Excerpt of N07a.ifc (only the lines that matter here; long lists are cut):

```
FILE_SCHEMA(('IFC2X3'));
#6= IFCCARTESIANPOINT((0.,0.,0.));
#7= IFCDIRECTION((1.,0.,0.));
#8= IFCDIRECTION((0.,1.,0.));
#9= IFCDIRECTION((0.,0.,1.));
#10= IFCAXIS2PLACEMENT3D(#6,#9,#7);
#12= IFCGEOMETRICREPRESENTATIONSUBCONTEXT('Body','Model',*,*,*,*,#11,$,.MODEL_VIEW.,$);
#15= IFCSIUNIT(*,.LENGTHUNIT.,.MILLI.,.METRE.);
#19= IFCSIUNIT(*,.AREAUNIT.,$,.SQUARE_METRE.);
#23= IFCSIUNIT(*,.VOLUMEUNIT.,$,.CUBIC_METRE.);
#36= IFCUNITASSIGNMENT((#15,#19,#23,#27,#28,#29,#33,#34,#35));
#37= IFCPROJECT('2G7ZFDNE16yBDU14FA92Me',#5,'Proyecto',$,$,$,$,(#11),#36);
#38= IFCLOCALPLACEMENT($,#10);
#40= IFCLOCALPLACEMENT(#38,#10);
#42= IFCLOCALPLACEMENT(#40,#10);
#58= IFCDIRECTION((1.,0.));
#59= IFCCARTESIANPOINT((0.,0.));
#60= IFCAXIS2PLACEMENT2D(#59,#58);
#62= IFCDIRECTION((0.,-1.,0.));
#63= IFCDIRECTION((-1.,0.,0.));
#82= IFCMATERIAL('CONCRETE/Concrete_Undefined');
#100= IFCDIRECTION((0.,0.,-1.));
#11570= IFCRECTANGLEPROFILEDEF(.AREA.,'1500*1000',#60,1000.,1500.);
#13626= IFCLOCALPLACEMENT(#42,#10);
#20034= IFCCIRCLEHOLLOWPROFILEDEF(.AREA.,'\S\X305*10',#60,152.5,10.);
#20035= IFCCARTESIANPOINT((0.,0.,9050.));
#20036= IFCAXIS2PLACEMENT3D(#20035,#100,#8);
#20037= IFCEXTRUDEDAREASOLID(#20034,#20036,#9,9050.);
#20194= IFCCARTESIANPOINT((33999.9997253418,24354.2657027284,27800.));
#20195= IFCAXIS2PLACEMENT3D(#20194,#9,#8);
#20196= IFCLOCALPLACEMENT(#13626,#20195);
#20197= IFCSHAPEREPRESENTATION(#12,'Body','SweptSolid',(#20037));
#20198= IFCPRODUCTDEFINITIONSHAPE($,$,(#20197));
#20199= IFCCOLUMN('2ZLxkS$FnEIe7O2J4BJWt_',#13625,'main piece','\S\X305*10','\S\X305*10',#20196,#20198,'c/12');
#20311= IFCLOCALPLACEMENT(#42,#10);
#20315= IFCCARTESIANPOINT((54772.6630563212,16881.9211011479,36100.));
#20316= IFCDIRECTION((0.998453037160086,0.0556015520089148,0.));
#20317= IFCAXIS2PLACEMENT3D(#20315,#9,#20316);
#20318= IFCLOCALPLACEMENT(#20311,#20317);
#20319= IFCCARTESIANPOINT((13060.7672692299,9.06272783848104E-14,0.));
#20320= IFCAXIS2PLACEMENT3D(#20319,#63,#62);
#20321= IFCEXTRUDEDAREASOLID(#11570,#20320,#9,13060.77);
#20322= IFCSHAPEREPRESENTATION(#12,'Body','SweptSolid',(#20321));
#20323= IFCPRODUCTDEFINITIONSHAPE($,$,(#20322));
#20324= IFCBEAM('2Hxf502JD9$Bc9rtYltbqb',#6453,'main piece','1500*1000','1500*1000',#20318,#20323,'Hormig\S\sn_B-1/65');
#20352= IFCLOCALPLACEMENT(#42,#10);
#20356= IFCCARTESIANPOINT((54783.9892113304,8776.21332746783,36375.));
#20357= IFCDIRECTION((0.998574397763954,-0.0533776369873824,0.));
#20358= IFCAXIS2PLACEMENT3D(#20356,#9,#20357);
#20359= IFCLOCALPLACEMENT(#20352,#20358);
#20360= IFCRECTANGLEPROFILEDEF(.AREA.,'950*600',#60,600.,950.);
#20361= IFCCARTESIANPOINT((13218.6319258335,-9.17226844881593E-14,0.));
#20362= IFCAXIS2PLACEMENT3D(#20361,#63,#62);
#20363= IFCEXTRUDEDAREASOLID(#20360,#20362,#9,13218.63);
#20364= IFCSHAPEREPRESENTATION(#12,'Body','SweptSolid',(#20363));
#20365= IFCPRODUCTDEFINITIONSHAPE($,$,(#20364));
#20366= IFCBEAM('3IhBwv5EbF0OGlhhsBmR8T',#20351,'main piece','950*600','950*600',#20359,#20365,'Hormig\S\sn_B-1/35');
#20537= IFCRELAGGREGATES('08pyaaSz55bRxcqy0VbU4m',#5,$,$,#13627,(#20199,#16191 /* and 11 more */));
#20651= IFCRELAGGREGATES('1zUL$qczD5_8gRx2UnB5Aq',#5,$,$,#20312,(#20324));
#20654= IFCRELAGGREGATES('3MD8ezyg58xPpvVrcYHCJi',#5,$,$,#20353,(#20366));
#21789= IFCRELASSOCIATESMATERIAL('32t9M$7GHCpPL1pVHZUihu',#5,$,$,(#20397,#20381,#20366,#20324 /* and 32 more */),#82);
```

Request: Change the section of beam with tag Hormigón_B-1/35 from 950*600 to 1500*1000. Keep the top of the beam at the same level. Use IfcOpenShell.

```python
import ifcopenshell
import ifcopenshell.util.element
import ifcopenshell.util.representation

model = ifcopenshell.open("N07a.ifc")

member = model.by_guid("3IhBwv5EbF0OGlhhsBmR8T")
source = next(p for p in model.by_type("IfcRectangleProfileDef") if p.ProfileName == "1500*1000")

body = ifcopenshell.util.representation.get_representation(member, "Model", "Body")
solid = body.Items[0]
old_profile = solid.SweptArea

# Copy the section's sizes but keep this member's own profile position.
profile = ifcopenshell.util.element.copy(model, source)
# Profiles are centred, so shift by half the change in depth to hold the top.
shift = (old_profile.YDim - profile.YDim) / 2
x, y = old_profile.Position.Location.Coordinates
up = (0.0, 1.0)  # upwards, in the solid's own plane
location = model.createIfcCartesianPoint((x + up[0] * shift, y + up[1] * shift))
profile.Position = model.createIfcAxis2Placement2D(location, old_profile.Position.RefDirection)
solid.SweptArea = profile
if not model.get_total_inverses(old_profile):
    ifcopenshell.util.element.remove_deep2(model, old_profile)
member.Description = member.Description.replace("950*600", "1500*1000")
member.ObjectType = member.ObjectType.replace("950*600", "1500*1000")

print(solid.SweptArea)

model.write("N07a_v2.ifc")
```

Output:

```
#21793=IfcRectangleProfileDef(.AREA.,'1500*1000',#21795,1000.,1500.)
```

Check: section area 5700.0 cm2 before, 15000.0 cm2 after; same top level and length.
